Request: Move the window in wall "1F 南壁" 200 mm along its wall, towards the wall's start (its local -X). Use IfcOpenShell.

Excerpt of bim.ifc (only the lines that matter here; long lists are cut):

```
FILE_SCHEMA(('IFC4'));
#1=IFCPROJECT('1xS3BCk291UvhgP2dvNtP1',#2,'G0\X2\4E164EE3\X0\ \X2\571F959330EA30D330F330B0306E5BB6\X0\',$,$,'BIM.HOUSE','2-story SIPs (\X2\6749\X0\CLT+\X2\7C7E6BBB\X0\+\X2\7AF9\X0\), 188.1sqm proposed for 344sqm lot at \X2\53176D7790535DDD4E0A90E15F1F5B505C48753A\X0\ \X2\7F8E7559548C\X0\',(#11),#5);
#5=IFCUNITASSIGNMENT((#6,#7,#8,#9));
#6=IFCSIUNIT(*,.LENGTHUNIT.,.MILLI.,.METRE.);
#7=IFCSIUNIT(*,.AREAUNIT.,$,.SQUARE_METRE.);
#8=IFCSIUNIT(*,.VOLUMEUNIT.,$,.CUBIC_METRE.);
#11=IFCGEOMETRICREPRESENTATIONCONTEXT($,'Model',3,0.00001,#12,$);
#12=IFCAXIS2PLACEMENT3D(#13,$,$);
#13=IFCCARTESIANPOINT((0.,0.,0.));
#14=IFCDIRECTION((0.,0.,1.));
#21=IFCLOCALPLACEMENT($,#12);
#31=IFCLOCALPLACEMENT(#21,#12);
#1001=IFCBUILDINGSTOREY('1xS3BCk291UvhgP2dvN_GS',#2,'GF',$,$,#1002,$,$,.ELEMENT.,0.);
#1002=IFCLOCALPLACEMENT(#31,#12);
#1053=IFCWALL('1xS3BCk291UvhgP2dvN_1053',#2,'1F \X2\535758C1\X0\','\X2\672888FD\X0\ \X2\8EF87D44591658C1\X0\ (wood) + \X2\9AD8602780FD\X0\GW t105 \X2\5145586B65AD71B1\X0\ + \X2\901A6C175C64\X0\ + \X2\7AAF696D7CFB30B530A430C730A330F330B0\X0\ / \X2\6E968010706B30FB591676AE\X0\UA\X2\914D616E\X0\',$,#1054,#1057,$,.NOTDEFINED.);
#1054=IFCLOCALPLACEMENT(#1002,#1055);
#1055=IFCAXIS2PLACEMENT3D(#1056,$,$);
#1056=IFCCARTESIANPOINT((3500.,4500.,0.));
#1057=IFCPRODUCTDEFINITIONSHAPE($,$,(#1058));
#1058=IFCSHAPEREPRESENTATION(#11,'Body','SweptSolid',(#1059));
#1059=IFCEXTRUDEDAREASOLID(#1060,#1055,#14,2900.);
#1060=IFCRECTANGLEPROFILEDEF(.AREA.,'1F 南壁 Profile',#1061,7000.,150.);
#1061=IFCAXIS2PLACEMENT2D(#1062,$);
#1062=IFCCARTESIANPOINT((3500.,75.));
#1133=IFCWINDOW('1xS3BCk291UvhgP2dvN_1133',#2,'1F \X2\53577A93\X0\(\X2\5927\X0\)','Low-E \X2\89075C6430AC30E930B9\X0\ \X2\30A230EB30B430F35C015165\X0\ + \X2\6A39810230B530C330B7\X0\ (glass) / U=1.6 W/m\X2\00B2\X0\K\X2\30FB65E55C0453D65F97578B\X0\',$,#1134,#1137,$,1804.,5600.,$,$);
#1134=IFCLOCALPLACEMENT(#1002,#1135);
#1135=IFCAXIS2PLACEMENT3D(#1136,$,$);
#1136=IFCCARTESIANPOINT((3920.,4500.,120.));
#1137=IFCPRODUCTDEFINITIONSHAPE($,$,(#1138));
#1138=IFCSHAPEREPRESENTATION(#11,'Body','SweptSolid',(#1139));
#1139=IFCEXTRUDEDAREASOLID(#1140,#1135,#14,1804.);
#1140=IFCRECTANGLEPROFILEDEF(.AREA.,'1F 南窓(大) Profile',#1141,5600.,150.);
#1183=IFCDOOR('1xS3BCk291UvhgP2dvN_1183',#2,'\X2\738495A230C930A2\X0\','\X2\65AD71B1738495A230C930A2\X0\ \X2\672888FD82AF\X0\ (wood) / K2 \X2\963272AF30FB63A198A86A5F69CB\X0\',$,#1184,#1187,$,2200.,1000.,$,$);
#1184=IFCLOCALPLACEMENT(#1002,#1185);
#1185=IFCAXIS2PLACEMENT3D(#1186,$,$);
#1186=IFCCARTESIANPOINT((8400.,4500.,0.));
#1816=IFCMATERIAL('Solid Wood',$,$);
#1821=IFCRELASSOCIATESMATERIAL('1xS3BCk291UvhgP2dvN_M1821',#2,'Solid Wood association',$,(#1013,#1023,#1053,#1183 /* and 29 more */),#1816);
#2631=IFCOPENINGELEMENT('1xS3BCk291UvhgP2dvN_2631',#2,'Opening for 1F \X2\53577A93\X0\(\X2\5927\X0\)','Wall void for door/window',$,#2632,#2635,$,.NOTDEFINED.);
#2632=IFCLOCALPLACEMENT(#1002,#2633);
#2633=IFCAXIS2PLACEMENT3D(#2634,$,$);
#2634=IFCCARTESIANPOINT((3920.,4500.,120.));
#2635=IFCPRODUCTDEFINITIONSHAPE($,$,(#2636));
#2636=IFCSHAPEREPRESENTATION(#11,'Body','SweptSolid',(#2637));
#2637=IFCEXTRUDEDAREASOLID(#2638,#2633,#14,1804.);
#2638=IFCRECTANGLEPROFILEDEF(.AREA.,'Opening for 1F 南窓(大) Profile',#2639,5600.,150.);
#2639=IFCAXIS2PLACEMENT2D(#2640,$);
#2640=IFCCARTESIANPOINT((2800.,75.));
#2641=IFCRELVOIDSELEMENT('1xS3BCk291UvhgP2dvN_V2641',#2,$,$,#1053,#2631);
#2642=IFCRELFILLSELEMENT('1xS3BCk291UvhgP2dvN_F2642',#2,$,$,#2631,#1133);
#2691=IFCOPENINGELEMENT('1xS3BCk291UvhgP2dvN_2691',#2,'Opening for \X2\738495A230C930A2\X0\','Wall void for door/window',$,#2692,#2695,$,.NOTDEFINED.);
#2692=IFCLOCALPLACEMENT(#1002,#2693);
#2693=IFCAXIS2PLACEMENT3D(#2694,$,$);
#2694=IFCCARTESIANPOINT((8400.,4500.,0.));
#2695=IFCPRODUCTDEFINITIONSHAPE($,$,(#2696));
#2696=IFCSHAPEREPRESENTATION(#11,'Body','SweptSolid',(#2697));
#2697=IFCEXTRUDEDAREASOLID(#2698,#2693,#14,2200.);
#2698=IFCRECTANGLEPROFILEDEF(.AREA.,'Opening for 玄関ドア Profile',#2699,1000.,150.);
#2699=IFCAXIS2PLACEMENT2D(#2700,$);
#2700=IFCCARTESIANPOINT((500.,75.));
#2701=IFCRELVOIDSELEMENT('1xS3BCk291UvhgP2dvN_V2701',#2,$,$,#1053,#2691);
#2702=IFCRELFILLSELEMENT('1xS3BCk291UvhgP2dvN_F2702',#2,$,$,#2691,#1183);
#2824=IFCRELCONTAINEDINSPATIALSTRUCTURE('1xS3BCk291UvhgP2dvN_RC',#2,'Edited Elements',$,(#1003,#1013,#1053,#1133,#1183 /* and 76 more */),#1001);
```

```python
import ifcopenshell
import ifcopenshell.api.geometry
import ifcopenshell.util.placement
import ifcopenshell.util.unit

model = ifcopenshell.open("bim.ifc")
unit_scale = ifcopenshell.util.unit.calculate_unit_scale(model)

window = model.by_id(1133)
opening = window.FillsVoids[0].RelatingOpeningElement
wall = opening.VoidsElements[0].RelatingBuildingElement

wall_matrix = ifcopenshell.util.placement.get_local_placement(wall.ObjectPlacement)
shift = wall_matrix[:3, 0] * -0.2 / unit_scale
before = ifcopenshell.util.placement.get_local_placement(window.ObjectPlacement)[:3, 3].copy()

# The window is not placed relative to its opening, so move both.
for product in (opening, window):
    matrix = ifcopenshell.util.placement.get_local_placement(product.ObjectPlacement)
    matrix[:3, 3] += shift
    ifcopenshell.api.geometry.edit_object_placement(model, product=product, matrix=matrix, is_si=False)

after = ifcopenshell.util.placement.get_local_placement(window.ObjectPlacement)[:3, 3]
print("window moved by", (after - before).round(3) + 0.0)

model.write("bim_rev.ifc")
```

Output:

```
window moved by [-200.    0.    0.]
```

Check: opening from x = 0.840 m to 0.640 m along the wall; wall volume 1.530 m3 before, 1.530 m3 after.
